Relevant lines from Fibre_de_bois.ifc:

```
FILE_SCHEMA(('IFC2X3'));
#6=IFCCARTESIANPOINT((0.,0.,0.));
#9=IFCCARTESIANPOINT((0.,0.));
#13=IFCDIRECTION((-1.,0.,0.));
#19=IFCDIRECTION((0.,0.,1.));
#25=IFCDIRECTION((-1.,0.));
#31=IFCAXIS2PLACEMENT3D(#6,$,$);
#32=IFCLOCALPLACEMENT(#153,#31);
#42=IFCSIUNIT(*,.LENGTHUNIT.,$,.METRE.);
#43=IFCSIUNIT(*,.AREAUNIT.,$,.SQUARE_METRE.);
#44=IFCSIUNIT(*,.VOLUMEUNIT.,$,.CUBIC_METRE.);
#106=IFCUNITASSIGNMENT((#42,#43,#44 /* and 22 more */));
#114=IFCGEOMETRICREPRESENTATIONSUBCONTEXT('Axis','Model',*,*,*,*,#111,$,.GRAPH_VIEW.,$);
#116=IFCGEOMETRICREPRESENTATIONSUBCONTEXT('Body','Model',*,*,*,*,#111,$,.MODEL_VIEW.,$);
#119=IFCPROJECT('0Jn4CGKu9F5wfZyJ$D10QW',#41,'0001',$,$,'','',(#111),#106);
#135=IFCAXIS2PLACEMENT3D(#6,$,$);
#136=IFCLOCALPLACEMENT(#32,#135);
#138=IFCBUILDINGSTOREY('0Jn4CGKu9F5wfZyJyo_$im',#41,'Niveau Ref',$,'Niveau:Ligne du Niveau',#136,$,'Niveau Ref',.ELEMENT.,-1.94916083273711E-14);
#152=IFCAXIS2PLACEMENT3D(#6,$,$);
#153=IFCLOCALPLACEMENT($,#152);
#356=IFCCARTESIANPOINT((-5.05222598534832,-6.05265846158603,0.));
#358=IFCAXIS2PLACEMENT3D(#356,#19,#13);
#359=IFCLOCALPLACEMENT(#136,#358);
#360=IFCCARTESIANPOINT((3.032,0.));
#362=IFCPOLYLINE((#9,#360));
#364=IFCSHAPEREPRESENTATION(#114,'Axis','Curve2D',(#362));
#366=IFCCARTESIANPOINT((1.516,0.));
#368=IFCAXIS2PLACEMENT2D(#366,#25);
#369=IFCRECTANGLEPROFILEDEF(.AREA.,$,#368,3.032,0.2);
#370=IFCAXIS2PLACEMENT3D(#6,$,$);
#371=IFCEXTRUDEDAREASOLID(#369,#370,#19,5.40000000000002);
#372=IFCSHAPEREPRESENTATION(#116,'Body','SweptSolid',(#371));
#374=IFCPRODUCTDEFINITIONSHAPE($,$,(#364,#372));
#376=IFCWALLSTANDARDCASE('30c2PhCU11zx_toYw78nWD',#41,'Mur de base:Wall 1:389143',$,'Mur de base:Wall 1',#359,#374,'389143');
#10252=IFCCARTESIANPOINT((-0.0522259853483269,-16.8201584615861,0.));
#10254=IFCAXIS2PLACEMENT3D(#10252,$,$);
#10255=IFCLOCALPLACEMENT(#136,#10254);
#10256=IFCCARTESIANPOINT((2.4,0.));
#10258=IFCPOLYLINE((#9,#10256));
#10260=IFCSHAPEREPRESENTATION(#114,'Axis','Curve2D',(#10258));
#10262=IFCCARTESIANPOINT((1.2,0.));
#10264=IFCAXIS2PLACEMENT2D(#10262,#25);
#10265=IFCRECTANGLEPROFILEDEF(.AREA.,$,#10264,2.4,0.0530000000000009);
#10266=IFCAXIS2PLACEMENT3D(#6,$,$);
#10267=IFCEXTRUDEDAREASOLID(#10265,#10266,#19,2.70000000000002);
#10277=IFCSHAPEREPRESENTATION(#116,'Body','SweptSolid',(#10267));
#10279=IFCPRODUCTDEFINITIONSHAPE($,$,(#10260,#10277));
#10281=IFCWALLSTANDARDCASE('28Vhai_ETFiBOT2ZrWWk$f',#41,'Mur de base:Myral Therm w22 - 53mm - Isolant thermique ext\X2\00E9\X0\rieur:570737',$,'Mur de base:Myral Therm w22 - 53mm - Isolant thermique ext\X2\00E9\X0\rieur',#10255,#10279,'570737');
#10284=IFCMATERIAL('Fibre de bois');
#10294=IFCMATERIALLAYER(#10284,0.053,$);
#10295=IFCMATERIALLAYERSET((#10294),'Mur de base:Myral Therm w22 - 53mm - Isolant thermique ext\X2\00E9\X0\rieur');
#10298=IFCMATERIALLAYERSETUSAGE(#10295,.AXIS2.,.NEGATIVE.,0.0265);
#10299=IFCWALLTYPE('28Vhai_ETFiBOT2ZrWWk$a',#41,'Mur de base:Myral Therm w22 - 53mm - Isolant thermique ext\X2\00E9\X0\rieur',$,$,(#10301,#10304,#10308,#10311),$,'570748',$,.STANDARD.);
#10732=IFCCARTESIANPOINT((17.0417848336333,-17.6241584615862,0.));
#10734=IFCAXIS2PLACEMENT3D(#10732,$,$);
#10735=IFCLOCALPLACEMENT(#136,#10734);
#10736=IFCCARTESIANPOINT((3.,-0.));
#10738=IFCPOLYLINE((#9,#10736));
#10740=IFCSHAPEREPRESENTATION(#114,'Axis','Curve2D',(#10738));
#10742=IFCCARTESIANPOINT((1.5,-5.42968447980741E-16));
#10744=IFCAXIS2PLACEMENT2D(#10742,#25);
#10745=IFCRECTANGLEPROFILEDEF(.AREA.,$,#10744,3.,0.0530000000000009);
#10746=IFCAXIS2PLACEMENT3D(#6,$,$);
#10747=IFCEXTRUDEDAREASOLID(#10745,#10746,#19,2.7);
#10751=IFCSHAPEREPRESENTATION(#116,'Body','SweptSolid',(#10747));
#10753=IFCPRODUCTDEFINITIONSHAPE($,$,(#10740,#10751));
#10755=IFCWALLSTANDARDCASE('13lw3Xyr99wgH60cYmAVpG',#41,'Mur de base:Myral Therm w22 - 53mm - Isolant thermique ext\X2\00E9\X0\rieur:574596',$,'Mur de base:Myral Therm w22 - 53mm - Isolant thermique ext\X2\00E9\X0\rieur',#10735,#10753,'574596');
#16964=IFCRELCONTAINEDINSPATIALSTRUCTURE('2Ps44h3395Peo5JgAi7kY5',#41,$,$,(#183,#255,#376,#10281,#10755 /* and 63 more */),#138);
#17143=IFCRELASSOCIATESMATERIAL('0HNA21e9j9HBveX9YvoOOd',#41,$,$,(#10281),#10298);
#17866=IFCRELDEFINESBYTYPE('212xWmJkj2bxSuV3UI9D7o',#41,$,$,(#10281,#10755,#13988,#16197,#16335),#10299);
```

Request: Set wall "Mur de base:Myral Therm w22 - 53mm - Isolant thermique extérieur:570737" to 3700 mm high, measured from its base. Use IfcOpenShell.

```python
import ifcopenshell
import ifcopenshell.geom
import ifcopenshell.util.representation
import ifcopenshell.util.shape
import ifcopenshell.util.unit

model = ifcopenshell.open("Fibre_de_bois.ifc")
unit_scale = ifcopenshell.util.unit.calculate_unit_scale(model)
settings = ifcopenshell.geom.settings()


def volume(element):
    """Net volume in cubic metres, openings subtracted."""
    shape = ifcopenshell.geom.create_shape(settings, element)
    return ifcopenshell.util.shape.get_volume(shape.geometry)


wall = model.by_id(10281)
before = volume(wall)

body = ifcopenshell.util.representation.get_representation(wall, "Model", "Body")
solid = body.Items[0]
old_height = solid.Depth
solid.Depth = 3.7 / unit_scale
after = volume(wall)

print(f"height {old_height:g} -> {solid.Depth:g}, volume {before:.3f} -> {after:.3f} m3")

model.write("Fibre_de_bois-out.ifc")
```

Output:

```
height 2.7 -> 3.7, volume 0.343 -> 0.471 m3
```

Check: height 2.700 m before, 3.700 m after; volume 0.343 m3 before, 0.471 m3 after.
